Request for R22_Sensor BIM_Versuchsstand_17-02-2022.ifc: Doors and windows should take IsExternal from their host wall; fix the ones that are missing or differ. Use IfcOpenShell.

First a look at what the model holds.

```python
import ifcopenshell
import ifcopenshell.util.element

model = ifcopenshell.open("R22_Sensor BIM_Versuchsstand_17-02-2022.ifc")
print(model.schema)
seen = {}
for e in model.by_type("IfcDoor") + model.by_type("IfcWindow"):
    if not e.FillsVoids:
        continue
    host = e.FillsVoids[0].RelatingOpeningElement.VoidsElements[0].RelatingBuildingElement
    own = ifcopenshell.util.element.get_pset(e, f"Pset_{e.is_a()[3:].removesuffix('StandardCase')}Common", "IsExternal")
    wall = ifcopenshell.util.element.get_pset(host, "Pset_WallCommon", "IsExternal")
    seen[e.is_a(), own, wall] = seen.get((e.is_a(), own, wall), 0) + 1
for (cls, own, wall), count in sorted(seen.items(), key=str):
    print(count, cls, "IsExternal:", own, "| host wall:", wall)
```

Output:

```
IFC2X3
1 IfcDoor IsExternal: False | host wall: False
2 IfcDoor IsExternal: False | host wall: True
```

```python
import ifcopenshell
import ifcopenshell.api.pset
import ifcopenshell.util.element

model = ifcopenshell.open("R22_Sensor BIM_Versuchsstand_17-02-2022.ifc")

count = 0
for ifc_class, pset_name in (("IfcDoor", "Pset_DoorCommon"), ("IfcWindow", "Pset_WindowCommon")):
    for e in model.by_type(ifc_class):
        if not e.FillsVoids:
            continue
        host = e.FillsVoids[0].RelatingOpeningElement.VoidsElements[0].RelatingBuildingElement
        external = ifcopenshell.util.element.get_pset(host, "Pset_WallCommon", "IsExternal")
        if external is None or ifcopenshell.util.element.get_pset(e, pset_name, "IsExternal") == external:
            continue
        pset = ifcopenshell.api.pset.add_pset(model, product=e, name=pset_name)
        ifcopenshell.api.pset.edit_pset(model, pset=pset, properties={"IsExternal": external})
        count += 1

print(count, "updated")

model.write("R22_Sensor BIM_Versuchsstand_17-02-2022-out.ifc")
```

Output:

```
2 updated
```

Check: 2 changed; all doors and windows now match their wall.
